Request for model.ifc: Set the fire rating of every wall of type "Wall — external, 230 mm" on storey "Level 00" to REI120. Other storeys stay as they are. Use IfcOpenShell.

First a look at what the model holds.

```python
import ifcopenshell
import ifcopenshell.util.element

model = ifcopenshell.open("model.ifc")
print(model.schema)
storey = next(s for s in model.by_type("IfcBuildingStorey") if s.Name == "Level 00")
walls = [e for e in ifcopenshell.util.element.get_decomposition(storey) if e.is_a("IfcWall")]
seen = {}
for e in walls:
    element_type = ifcopenshell.util.element.get_type(e)
    key = (element_type.Name if element_type != e and element_type else None, ifcopenshell.util.element.get_pset(e, "Pset_WallCommon", "FireRating"))
    seen[key] = seen.get(key, 0) + 1
for (name, value), count in sorted(seen.items(), key=str):
    print(count, "x", name, "|", value)
```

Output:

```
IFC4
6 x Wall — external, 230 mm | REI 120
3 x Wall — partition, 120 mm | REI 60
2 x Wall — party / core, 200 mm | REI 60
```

```python
import ifcopenshell
import ifcopenshell.api.pset
import ifcopenshell.util.element

model = ifcopenshell.open("model.ifc")

storey = next(s for s in model.by_type("IfcBuildingStorey") if s.Name == "Level 00")
walls = [e for e in ifcopenshell.util.element.get_decomposition(storey) if e.is_a("IfcWall")]

count = 0
for e in walls:
    element_type = ifcopenshell.util.element.get_type(e)
    if element_type in (None, e) or element_type.Name != "Wall — external, 230 mm":
        continue
    # add_pset returns the element's existing set when there is one.
    pset = ifcopenshell.api.pset.add_pset(model, product=e, name="Pset_WallCommon")
    ifcopenshell.api.pset.edit_pset(model, pset=pset, properties={"FireRating": "REI120"})
    count += 1

print(count, "walls updated")

model.write("model-out.ifc")
```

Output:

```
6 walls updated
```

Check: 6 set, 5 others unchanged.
